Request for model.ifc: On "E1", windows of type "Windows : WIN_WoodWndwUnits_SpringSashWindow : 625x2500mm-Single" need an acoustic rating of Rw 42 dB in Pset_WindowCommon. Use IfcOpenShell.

First a look at what the model holds.

```python
import ifcopenshell
import ifcopenshell.util.element

model = ifcopenshell.open("model.ifc")
print(model.schema)
storey = next(s for s in model.by_type("IfcBuildingStorey") if s.Name == "E1")
windows = [e for e in ifcopenshell.util.element.get_decomposition(storey) if e.is_a("IfcWindow")]
seen = {}
for e in windows:
    element_type = ifcopenshell.util.element.get_type(e)
    key = (element_type.Name if element_type != e and element_type else None, ifcopenshell.util.element.get_pset(e, "Pset_WindowCommon", "AcousticRating"))
    seen[key] = seen.get(key, 0) + 1
for (name, value), count in sorted(seen.items(), key=str):
    print(count, "x", name, "|", value)
```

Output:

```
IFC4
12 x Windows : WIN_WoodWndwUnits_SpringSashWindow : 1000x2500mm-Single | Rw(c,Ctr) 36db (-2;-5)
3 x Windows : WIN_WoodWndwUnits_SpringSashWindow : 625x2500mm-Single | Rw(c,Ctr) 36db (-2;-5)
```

```python
import ifcopenshell
import ifcopenshell.api.pset
import ifcopenshell.util.element

model = ifcopenshell.open("model.ifc")

storey = next(s for s in model.by_type("IfcBuildingStorey") if s.Name == "E1")
windows = [e for e in ifcopenshell.util.element.get_decomposition(storey) if e.is_a("IfcWindow")]

count = 0
for e in windows:
    element_type = ifcopenshell.util.element.get_type(e)
    if element_type in (None, e) or element_type.Name != "Windows : WIN_WoodWndwUnits_SpringSashWindow : 625x2500mm-Single":
        continue
    # add_pset returns the element's existing set when there is one.
    pset = ifcopenshell.api.pset.add_pset(model, product=e, name="Pset_WindowCommon")
    ifcopenshell.api.pset.edit_pset(model, pset=pset, properties={"AcousticRating": "Rw 42 dB"})
    count += 1

print(count, "windows updated")

model.write("model-out.ifc")
```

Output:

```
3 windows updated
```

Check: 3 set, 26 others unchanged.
